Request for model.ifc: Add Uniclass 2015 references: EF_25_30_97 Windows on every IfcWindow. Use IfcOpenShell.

First a look at what the model holds.

```python
import ifcopenshell

model = ifcopenshell.open("model.ifc")
print(model.schema)
print("classifications:", [c.Name for c in model.by_type("IfcClassification")])
for ifc_class in ("IfcDoor", "IfcRoof", "IfcStair", "IfcWall", "IfcWindow"):
    print(ifc_class, len(model.by_type(ifc_class)))
```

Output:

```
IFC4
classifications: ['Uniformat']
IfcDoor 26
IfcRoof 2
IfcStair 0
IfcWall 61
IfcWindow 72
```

```python
import ifcopenshell
import ifcopenshell.api.classification

model = ifcopenshell.open("model.ifc")

system = ifcopenshell.api.classification.add_classification(model, classification="Uniclass 2015")

codes = {
    "IfcWindow": ("EF_25_30_97", "Windows"),
}
for ifc_class, (code, name) in codes.items():
    products = model.by_type(ifc_class)
    ifcopenshell.api.classification.add_reference(
        model, products=products, classification=system, identification=code, name=name
    )
    print(code, len(products))

model.write("model_rev.ifc")
```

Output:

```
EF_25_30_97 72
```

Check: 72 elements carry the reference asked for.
